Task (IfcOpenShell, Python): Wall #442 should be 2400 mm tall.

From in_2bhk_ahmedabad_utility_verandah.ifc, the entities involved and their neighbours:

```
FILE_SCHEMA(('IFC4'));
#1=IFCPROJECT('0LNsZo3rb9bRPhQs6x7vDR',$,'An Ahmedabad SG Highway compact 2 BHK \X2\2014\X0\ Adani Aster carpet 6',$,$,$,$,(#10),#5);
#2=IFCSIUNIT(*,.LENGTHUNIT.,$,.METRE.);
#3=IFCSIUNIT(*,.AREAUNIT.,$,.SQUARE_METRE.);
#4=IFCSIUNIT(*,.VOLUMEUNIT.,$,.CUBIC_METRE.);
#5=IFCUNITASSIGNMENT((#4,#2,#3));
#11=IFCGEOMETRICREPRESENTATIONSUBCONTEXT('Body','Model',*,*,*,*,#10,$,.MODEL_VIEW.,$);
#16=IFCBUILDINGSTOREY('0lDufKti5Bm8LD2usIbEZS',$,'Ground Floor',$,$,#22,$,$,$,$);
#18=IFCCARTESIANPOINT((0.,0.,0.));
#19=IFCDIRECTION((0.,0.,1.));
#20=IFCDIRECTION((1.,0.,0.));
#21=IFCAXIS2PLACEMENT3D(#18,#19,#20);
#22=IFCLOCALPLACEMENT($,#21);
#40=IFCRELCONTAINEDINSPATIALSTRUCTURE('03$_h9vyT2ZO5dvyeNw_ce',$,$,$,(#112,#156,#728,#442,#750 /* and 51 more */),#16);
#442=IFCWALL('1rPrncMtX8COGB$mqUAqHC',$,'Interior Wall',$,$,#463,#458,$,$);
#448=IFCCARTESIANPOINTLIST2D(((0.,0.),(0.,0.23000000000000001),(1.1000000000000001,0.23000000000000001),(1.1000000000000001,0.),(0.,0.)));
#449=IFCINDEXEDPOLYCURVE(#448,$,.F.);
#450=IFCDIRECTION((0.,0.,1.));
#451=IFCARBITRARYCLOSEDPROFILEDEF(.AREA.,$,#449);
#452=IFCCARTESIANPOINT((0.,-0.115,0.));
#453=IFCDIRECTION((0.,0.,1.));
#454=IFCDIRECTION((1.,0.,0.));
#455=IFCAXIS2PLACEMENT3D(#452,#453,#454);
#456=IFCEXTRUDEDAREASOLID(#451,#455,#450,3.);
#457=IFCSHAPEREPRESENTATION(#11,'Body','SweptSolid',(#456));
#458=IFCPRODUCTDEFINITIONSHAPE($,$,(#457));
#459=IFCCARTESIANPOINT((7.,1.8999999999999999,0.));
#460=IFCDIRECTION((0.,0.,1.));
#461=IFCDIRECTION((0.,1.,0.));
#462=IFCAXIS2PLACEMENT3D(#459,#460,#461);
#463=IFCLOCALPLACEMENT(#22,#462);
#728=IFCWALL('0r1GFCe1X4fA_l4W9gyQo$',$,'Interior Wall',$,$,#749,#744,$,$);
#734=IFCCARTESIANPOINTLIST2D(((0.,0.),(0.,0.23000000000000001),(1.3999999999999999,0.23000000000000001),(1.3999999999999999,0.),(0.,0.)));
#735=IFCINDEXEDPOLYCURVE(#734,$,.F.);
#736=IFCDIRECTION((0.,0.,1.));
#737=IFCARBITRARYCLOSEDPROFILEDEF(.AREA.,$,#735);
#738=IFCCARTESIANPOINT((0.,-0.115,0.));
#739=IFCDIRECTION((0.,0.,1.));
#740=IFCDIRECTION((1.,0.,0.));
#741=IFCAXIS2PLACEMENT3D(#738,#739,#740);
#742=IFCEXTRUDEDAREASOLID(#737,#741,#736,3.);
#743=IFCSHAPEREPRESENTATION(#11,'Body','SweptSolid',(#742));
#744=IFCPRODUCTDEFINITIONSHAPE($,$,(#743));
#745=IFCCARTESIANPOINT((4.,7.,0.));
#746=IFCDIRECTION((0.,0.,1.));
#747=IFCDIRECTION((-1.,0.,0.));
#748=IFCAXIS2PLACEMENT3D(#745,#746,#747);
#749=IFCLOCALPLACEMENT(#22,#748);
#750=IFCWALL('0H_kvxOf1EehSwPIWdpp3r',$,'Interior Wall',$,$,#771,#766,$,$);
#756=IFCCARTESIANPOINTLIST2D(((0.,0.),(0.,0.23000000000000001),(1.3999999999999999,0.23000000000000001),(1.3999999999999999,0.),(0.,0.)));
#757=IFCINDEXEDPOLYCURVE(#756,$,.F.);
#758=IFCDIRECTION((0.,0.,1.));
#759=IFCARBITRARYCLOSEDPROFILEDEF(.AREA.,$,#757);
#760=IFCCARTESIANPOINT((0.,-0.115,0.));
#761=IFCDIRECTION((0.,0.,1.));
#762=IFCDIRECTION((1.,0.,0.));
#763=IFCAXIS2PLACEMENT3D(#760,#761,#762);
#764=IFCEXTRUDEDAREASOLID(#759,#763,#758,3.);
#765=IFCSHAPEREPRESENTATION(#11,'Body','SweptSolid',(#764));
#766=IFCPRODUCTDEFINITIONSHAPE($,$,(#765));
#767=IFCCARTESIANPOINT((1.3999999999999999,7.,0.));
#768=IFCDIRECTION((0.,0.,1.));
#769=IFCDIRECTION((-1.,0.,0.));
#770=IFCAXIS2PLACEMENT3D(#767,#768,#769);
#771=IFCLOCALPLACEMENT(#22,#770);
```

```python
import ifcopenshell
import ifcopenshell.geom
import ifcopenshell.util.representation
import ifcopenshell.util.shape

model = ifcopenshell.open("in_2bhk_ahmedabad_utility_verandah.ifc")
settings = ifcopenshell.geom.settings()


def volume(element):
    """Net volume in cubic metres, openings subtracted."""
    shape = ifcopenshell.geom.create_shape(settings, element)
    return ifcopenshell.util.shape.get_volume(shape.geometry)


wall = model.by_guid("1rPrncMtX8COGB$mqUAqHC")
before = volume(wall)

body = ifcopenshell.util.representation.get_representation(wall, "Model", "Body")
solid = body.Items[0]
old_height = solid.Depth
solid.Depth = 2.4
after = volume(wall)

print(f"height {old_height:g} -> {solid.Depth:g}, volume {before:.3f} -> {after:.3f} m3")

model.write("in_2bhk_ahmedabad_utility_verandah_updated.ifc")
```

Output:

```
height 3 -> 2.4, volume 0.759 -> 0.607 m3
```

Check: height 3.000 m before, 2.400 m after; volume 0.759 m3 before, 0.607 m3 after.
